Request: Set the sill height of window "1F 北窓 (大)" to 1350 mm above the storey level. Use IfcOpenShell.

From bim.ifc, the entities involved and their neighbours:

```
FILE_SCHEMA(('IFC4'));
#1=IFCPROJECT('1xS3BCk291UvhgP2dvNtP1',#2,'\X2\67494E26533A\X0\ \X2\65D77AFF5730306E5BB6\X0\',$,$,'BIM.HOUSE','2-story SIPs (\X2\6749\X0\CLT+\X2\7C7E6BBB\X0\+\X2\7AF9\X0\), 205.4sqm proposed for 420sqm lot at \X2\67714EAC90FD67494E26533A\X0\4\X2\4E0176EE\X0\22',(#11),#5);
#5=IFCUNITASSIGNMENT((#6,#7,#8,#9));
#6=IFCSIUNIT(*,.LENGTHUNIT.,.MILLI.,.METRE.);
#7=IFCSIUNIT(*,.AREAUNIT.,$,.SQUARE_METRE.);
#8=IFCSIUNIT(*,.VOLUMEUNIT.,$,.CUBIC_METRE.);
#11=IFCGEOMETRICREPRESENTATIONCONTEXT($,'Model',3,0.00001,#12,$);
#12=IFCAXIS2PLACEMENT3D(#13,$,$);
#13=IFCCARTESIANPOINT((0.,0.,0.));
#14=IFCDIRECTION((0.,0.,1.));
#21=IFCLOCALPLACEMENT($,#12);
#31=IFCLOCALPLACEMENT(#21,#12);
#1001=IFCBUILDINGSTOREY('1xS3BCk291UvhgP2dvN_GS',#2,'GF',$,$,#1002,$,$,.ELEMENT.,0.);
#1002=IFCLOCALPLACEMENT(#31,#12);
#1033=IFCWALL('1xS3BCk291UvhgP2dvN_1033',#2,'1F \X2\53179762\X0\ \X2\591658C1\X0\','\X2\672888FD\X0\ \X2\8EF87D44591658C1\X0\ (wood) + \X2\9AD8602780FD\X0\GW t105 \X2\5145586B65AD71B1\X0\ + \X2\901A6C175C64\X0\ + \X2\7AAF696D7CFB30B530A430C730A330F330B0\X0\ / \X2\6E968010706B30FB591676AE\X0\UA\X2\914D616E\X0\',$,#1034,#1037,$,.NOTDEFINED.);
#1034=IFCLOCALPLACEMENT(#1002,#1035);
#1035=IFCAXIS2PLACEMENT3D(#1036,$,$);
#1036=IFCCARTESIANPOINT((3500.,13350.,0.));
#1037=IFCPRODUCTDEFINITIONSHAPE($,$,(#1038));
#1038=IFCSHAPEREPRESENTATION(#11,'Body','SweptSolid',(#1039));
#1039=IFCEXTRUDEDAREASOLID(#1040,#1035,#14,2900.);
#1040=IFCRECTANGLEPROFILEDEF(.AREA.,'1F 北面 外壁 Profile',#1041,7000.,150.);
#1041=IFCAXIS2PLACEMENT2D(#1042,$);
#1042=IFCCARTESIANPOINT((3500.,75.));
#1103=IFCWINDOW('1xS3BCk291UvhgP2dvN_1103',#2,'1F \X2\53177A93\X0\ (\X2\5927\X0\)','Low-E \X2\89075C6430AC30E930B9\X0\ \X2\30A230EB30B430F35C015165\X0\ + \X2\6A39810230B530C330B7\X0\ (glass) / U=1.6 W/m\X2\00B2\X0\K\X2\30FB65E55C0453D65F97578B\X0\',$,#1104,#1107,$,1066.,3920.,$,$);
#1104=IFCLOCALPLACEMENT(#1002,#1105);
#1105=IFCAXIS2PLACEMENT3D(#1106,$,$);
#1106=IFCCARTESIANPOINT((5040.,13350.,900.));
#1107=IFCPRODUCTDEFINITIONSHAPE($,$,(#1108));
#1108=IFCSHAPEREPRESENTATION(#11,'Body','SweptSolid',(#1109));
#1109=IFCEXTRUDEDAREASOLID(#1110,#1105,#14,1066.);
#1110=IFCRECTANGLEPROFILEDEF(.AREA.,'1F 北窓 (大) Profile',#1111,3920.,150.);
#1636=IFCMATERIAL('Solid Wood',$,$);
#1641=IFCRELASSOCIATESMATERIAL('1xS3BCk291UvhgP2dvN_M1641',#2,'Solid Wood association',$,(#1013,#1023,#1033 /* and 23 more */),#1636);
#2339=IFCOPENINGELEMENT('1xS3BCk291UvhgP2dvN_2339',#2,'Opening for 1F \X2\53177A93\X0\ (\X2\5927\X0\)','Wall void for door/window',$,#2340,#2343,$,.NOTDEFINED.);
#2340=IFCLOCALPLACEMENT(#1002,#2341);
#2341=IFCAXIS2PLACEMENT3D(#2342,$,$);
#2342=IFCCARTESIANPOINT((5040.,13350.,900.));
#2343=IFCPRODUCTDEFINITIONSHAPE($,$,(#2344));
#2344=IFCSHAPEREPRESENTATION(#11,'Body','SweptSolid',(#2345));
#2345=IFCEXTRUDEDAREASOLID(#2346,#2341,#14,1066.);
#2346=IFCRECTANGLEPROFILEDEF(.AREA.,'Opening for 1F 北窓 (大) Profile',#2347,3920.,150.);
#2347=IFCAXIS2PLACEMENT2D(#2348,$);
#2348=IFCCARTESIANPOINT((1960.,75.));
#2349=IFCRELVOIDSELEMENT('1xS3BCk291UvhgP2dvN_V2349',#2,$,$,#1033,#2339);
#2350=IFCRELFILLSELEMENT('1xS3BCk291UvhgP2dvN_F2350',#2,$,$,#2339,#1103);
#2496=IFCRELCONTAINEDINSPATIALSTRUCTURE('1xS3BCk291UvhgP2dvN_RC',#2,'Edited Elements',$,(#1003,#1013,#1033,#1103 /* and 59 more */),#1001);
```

```python
import numpy as np
import ifcopenshell
import ifcopenshell.api.geometry
import ifcopenshell.geom
import ifcopenshell.util.element
import ifcopenshell.util.placement
import ifcopenshell.util.shape
import ifcopenshell.util.unit

model = ifcopenshell.open("bim.ifc")
unit_scale = ifcopenshell.util.unit.calculate_unit_scale(model)

window = model.by_guid("1xS3BCk291UvhgP2dvN_1103")
opening = window.FillsVoids[0].RelatingOpeningElement
storey = ifcopenshell.util.element.get_container(window, ifc_class="IfcBuildingStorey")
level = ifcopenshell.util.placement.get_local_placement(storey.ObjectPlacement)[2, 3]

# The opening's origin need not be at the sill, so measure its lowest point.
shape = ifcopenshell.geom.create_shape(ifcopenshell.geom.settings(), opening)
bottom = ifcopenshell.util.shape.get_shape_bottom_elevation(shape, shape.geometry) / unit_scale
dz = level + 1.35 / unit_scale - bottom

shift = np.array([0.0, 0.0, dz])
# The window is not placed relative to its opening, so move both.
for product in (opening, window):
    matrix = ifcopenshell.util.placement.get_local_placement(product.ObjectPlacement)
    matrix[:3, 3] += shift
    ifcopenshell.api.geometry.edit_object_placement(model, product=product, matrix=matrix, is_si=False)

print(f"moved by {dz * unit_scale:+.3f} m")

model.write("bim_edited.ifc")
```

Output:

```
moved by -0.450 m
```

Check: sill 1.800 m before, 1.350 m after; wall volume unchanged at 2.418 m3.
